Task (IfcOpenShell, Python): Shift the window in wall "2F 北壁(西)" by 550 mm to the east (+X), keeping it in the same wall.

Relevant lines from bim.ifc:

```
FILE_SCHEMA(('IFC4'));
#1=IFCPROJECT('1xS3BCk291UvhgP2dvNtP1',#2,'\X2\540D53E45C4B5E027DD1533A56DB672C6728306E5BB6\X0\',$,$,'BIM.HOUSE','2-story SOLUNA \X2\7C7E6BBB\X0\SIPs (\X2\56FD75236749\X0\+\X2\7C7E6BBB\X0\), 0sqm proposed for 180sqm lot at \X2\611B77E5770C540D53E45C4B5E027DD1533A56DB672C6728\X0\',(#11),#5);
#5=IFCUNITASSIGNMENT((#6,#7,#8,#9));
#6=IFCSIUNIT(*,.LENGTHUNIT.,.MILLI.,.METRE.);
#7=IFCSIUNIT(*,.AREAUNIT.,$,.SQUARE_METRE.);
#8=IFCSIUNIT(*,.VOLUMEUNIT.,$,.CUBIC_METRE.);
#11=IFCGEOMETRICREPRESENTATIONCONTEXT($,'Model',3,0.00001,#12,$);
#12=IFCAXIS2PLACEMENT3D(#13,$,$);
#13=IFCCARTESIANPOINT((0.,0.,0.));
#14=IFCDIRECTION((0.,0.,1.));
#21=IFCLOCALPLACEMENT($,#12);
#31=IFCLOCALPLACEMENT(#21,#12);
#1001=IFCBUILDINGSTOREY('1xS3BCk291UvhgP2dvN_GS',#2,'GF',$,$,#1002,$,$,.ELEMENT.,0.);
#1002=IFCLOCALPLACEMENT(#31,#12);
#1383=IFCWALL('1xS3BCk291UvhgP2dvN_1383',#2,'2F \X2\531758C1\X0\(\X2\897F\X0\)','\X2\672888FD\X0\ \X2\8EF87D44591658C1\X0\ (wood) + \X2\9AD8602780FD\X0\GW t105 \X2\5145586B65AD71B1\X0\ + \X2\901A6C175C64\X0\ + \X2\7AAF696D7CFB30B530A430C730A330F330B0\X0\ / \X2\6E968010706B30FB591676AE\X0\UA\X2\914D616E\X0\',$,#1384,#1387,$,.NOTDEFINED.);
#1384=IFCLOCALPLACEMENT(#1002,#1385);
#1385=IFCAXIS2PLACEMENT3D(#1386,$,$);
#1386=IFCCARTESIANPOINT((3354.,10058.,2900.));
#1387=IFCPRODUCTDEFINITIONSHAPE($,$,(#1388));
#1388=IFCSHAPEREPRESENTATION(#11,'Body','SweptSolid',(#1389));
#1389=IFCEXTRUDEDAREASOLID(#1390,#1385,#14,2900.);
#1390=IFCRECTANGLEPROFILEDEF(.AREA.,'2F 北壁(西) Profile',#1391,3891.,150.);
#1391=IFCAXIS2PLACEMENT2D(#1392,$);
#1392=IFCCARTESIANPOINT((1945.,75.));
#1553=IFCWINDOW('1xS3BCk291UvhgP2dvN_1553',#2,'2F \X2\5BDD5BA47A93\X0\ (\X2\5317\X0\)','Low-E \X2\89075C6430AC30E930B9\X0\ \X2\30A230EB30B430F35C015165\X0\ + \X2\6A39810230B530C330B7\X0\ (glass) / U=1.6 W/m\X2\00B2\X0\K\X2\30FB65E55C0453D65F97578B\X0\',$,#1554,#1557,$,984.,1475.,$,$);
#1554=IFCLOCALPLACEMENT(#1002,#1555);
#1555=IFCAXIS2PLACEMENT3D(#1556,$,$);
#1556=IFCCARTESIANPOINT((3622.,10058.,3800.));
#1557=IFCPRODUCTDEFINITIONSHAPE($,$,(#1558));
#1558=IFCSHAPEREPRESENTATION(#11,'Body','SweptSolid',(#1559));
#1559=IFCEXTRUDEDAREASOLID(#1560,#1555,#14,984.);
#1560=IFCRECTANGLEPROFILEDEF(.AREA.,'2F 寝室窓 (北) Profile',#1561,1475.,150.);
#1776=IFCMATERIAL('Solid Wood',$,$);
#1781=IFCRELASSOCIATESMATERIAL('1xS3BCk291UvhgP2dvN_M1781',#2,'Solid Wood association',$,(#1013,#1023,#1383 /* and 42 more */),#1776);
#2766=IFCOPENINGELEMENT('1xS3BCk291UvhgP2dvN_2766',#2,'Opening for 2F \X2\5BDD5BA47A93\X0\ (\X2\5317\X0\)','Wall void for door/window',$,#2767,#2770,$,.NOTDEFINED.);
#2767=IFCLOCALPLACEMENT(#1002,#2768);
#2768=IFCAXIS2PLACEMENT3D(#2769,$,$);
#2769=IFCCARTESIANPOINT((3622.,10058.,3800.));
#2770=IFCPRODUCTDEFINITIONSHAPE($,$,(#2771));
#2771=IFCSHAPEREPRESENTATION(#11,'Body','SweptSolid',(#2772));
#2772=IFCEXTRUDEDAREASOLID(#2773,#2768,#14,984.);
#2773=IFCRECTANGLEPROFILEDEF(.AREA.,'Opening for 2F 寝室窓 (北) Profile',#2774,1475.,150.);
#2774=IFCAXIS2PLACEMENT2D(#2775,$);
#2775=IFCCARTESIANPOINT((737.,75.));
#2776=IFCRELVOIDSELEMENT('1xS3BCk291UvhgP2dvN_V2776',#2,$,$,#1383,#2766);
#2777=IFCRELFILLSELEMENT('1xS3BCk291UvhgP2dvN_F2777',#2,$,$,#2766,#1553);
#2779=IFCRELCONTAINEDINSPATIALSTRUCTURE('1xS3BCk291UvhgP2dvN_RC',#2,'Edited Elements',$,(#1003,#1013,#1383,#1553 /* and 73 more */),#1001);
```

```python
import ifcopenshell
import ifcopenshell.api.geometry
import ifcopenshell.util.placement
import ifcopenshell.util.unit

model = ifcopenshell.open("bim.ifc")
unit_scale = ifcopenshell.util.unit.calculate_unit_scale(model)

window = model.by_id(1553)
opening = window.FillsVoids[0].RelatingOpeningElement
wall = opening.VoidsElements[0].RelatingBuildingElement

wall_matrix = ifcopenshell.util.placement.get_local_placement(wall.ObjectPlacement)
shift = wall_matrix[:3, 0] * 0.55 / unit_scale
before = ifcopenshell.util.placement.get_local_placement(window.ObjectPlacement)[:3, 3].copy()

# The window is not placed relative to its opening, so move both.
for product in (opening, window):
    matrix = ifcopenshell.util.placement.get_local_placement(product.ObjectPlacement)
    matrix[:3, 3] += shift
    ifcopenshell.api.geometry.edit_object_placement(model, product=product, matrix=matrix, is_si=False)

after = ifcopenshell.util.placement.get_local_placement(window.ObjectPlacement)[:3, 3]
print("window moved by", (after - before).round(3) + 0.0)

model.write("bim_edited.ifc")
```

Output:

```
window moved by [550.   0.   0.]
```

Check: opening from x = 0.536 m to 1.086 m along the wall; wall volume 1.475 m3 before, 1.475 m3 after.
